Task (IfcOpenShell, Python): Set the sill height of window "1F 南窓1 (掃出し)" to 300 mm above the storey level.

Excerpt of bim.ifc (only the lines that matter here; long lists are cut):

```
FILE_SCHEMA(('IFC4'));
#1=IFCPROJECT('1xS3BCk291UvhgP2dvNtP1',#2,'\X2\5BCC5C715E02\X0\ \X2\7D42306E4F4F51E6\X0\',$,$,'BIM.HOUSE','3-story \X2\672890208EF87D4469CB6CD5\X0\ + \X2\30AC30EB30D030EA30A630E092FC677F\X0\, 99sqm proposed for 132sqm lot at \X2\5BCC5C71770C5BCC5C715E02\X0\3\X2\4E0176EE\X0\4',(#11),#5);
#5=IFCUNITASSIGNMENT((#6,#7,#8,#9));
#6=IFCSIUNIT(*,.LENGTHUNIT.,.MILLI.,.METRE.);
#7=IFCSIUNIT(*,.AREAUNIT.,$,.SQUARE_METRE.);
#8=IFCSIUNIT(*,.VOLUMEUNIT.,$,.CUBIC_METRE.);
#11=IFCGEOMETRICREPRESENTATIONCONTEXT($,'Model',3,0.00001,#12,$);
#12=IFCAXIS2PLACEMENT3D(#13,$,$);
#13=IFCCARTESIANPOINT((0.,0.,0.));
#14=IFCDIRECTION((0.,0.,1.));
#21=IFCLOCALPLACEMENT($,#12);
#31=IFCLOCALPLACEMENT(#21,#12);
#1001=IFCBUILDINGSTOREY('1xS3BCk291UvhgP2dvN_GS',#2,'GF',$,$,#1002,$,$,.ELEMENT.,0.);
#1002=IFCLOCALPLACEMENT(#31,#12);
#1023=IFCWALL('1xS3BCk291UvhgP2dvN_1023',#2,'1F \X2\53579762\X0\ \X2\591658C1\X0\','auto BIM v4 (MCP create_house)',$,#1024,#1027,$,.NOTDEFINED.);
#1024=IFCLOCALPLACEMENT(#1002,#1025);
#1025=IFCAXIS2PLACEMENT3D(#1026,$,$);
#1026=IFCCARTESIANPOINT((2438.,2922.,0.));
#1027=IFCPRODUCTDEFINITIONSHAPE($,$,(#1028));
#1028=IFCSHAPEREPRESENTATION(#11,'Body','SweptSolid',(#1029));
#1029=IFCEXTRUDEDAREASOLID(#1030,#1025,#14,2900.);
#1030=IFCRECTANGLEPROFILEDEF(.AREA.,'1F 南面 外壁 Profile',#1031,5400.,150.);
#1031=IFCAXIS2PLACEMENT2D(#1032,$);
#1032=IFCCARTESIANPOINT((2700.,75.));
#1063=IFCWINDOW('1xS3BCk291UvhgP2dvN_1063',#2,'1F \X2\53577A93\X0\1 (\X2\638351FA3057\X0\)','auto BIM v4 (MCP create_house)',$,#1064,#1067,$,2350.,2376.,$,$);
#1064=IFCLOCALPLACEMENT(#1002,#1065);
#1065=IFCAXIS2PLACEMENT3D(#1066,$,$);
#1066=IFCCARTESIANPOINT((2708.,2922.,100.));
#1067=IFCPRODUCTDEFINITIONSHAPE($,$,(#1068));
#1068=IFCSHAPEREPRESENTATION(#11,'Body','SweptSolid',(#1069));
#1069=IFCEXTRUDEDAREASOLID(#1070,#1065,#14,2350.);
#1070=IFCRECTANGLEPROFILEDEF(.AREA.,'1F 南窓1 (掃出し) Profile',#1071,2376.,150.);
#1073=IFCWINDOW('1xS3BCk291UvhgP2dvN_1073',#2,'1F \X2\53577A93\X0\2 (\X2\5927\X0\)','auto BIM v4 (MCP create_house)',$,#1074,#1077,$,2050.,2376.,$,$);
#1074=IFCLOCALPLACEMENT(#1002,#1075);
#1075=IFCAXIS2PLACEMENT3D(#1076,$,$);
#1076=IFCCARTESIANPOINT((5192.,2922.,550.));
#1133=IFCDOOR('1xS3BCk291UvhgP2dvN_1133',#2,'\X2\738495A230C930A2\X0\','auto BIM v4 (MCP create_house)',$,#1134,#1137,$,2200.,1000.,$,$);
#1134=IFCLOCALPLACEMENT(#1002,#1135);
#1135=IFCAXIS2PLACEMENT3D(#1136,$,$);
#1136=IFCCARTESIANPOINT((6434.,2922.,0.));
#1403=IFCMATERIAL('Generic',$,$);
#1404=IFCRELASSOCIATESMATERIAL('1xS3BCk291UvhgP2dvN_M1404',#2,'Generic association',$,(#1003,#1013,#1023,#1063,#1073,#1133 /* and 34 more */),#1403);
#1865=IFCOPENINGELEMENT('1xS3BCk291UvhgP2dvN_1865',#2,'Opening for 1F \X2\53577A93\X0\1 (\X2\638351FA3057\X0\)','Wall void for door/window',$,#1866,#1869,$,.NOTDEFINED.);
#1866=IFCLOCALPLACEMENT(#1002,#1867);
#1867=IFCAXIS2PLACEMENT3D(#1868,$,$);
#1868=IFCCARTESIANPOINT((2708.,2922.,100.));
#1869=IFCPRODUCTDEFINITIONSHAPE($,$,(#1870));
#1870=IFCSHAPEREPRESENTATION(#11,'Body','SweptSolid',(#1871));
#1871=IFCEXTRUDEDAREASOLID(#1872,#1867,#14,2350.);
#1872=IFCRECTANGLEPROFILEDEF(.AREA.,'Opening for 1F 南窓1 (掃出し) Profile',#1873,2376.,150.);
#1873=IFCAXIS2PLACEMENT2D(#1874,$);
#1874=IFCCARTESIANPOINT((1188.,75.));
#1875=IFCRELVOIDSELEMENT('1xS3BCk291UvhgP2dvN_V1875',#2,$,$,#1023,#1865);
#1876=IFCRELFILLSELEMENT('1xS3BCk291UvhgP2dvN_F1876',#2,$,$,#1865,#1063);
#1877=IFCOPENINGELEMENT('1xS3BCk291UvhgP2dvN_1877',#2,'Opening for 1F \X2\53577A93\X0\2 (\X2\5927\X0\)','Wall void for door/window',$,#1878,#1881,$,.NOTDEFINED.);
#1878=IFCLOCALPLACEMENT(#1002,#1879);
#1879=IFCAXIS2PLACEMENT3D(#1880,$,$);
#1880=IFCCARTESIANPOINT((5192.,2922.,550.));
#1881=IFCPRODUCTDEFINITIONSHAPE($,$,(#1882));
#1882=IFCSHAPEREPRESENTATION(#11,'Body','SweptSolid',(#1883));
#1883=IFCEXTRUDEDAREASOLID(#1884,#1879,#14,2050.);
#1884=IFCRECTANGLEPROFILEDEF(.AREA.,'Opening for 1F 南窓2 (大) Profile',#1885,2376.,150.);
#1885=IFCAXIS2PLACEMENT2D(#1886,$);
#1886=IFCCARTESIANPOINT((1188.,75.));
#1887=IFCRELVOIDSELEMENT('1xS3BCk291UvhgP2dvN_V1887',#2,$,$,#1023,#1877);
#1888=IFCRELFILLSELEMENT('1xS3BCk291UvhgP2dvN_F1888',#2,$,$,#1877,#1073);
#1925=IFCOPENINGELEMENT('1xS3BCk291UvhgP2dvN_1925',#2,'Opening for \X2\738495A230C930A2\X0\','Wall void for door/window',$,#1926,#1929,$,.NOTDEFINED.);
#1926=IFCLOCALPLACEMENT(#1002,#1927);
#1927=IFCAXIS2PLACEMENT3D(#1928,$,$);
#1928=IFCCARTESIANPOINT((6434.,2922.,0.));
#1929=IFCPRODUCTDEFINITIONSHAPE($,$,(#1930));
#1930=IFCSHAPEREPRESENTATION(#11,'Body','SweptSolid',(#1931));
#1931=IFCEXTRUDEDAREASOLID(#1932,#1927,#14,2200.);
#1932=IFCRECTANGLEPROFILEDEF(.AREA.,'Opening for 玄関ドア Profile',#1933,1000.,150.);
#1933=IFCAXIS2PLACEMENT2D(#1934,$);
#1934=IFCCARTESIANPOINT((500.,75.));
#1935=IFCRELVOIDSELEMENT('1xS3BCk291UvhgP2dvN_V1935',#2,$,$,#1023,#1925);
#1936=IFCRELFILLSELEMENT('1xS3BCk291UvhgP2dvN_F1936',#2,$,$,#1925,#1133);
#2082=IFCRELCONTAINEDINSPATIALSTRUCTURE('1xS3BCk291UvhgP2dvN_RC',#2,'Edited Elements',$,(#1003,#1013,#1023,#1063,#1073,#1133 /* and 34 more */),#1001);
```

```python
import numpy as np
import ifcopenshell
import ifcopenshell.api.geometry
import ifcopenshell.geom
import ifcopenshell.util.element
import ifcopenshell.util.placement
import ifcopenshell.util.shape
import ifcopenshell.util.unit

model = ifcopenshell.open("bim.ifc")
unit_scale = ifcopenshell.util.unit.calculate_unit_scale(model)

window = model.by_guid("1xS3BCk291UvhgP2dvN_1063")
opening = window.FillsVoids[0].RelatingOpeningElement
storey = ifcopenshell.util.element.get_container(window, ifc_class="IfcBuildingStorey")
level = ifcopenshell.util.placement.get_local_placement(storey.ObjectPlacement)[2, 3]

# The opening's origin need not be at the sill, so measure its lowest point.
shape = ifcopenshell.geom.create_shape(ifcopenshell.geom.settings(), opening)
bottom = ifcopenshell.util.shape.get_shape_bottom_elevation(shape, shape.geometry) / unit_scale
dz = level + 0.3 / unit_scale - bottom

shift = np.array([0.0, 0.0, dz])
# The window is not placed relative to its opening, so move both.
for product in (opening, window):
    matrix = ifcopenshell.util.placement.get_local_placement(product.ObjectPlacement)
    matrix[:3, 3] += shift
    ifcopenshell.api.geometry.edit_object_placement(model, product=product, matrix=matrix, is_si=False)

print(f"moved by {dz * unit_scale:+.3f} m")

model.write("bim_edited.ifc")
```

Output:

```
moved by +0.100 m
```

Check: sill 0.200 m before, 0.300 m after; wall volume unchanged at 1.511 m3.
